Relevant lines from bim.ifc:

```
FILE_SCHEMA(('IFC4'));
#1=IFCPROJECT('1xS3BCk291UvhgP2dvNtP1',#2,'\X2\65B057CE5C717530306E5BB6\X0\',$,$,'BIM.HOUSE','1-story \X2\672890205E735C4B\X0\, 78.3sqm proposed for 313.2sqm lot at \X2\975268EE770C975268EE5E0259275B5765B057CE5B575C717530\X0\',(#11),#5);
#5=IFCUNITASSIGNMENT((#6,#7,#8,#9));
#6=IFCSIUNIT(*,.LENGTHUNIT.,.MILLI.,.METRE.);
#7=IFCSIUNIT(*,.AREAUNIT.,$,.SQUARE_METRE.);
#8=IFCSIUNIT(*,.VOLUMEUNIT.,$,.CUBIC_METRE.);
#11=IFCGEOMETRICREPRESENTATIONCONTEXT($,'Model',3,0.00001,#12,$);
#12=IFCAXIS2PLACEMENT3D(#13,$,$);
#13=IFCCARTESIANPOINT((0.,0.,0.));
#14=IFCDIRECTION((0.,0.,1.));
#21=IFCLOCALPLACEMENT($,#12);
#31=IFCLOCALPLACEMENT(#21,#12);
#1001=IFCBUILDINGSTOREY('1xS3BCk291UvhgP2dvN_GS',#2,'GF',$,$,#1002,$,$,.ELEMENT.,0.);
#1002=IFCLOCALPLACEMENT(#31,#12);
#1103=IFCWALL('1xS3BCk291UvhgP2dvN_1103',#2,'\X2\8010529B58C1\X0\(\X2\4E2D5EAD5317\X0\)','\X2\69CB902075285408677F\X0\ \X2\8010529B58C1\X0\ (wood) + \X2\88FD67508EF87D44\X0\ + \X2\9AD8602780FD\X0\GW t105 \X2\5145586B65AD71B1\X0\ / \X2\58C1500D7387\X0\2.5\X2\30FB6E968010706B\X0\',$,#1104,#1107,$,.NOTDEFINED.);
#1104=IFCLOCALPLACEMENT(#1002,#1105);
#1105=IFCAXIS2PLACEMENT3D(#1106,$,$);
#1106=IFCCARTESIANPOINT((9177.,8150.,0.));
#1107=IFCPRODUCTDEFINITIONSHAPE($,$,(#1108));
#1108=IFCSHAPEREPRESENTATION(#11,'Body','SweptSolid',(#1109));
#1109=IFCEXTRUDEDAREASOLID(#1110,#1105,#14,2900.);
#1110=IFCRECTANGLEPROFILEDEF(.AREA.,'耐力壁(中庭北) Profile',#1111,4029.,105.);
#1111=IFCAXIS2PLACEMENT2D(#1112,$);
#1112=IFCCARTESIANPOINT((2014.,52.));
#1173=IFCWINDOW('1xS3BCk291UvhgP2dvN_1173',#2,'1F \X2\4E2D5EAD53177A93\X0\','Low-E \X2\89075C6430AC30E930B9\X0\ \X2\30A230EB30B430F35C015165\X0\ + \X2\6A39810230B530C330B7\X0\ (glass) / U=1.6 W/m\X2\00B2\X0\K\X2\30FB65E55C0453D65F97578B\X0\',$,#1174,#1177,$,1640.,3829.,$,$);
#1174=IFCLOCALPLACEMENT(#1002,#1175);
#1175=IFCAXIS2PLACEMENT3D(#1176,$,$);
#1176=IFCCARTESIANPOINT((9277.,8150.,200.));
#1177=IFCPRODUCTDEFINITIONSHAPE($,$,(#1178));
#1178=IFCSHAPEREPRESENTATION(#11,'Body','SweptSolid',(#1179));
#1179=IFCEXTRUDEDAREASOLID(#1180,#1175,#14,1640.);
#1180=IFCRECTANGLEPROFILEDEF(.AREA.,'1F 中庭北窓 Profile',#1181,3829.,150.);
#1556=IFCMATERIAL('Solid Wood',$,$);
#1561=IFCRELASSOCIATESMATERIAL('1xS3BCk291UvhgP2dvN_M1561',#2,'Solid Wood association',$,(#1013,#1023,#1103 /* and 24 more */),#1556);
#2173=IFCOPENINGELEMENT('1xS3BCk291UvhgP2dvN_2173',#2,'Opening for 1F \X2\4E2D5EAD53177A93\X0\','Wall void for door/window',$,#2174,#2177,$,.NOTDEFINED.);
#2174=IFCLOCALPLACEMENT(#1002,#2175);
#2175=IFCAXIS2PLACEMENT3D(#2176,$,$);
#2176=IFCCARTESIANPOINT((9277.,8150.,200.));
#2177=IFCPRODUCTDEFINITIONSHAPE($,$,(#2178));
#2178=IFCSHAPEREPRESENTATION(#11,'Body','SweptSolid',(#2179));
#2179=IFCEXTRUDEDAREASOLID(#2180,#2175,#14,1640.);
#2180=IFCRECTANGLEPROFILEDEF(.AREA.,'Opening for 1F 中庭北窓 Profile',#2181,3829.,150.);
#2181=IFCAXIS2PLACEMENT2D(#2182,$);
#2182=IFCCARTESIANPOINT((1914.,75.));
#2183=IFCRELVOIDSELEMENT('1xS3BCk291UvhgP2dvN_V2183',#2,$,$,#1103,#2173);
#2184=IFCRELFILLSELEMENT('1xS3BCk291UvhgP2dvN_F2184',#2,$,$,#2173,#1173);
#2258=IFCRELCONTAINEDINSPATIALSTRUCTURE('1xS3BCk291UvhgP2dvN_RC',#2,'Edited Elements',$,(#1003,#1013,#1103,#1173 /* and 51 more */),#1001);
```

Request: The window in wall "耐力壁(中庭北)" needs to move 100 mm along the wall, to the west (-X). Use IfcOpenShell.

```python
import ifcopenshell
import ifcopenshell.api.geometry
import ifcopenshell.util.placement
import ifcopenshell.util.unit

model = ifcopenshell.open("bim.ifc")
unit_scale = ifcopenshell.util.unit.calculate_unit_scale(model)

window = model.by_guid("1xS3BCk291UvhgP2dvN_1173")
opening = window.FillsVoids[0].RelatingOpeningElement
wall = opening.VoidsElements[0].RelatingBuildingElement

wall_matrix = ifcopenshell.util.placement.get_local_placement(wall.ObjectPlacement)
shift = wall_matrix[:3, 0] * -0.1 / unit_scale
before = ifcopenshell.util.placement.get_local_placement(window.ObjectPlacement)[:3, 3].copy()

# The window is not placed relative to its opening, so move both.
for product in (opening, window):
    matrix = ifcopenshell.util.placement.get_local_placement(product.ObjectPlacement)
    matrix[:3, 3] += shift
    ifcopenshell.api.geometry.edit_object_placement(model, product=product, matrix=matrix, is_si=False)

after = ifcopenshell.util.placement.get_local_placement(window.ObjectPlacement)[:3, 3]
print("window moved by", (after - before).round(3) + 0.0)

model.write("bim_v2.ifc")
```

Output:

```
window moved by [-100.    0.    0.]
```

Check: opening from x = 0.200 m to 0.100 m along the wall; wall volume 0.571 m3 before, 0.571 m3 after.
